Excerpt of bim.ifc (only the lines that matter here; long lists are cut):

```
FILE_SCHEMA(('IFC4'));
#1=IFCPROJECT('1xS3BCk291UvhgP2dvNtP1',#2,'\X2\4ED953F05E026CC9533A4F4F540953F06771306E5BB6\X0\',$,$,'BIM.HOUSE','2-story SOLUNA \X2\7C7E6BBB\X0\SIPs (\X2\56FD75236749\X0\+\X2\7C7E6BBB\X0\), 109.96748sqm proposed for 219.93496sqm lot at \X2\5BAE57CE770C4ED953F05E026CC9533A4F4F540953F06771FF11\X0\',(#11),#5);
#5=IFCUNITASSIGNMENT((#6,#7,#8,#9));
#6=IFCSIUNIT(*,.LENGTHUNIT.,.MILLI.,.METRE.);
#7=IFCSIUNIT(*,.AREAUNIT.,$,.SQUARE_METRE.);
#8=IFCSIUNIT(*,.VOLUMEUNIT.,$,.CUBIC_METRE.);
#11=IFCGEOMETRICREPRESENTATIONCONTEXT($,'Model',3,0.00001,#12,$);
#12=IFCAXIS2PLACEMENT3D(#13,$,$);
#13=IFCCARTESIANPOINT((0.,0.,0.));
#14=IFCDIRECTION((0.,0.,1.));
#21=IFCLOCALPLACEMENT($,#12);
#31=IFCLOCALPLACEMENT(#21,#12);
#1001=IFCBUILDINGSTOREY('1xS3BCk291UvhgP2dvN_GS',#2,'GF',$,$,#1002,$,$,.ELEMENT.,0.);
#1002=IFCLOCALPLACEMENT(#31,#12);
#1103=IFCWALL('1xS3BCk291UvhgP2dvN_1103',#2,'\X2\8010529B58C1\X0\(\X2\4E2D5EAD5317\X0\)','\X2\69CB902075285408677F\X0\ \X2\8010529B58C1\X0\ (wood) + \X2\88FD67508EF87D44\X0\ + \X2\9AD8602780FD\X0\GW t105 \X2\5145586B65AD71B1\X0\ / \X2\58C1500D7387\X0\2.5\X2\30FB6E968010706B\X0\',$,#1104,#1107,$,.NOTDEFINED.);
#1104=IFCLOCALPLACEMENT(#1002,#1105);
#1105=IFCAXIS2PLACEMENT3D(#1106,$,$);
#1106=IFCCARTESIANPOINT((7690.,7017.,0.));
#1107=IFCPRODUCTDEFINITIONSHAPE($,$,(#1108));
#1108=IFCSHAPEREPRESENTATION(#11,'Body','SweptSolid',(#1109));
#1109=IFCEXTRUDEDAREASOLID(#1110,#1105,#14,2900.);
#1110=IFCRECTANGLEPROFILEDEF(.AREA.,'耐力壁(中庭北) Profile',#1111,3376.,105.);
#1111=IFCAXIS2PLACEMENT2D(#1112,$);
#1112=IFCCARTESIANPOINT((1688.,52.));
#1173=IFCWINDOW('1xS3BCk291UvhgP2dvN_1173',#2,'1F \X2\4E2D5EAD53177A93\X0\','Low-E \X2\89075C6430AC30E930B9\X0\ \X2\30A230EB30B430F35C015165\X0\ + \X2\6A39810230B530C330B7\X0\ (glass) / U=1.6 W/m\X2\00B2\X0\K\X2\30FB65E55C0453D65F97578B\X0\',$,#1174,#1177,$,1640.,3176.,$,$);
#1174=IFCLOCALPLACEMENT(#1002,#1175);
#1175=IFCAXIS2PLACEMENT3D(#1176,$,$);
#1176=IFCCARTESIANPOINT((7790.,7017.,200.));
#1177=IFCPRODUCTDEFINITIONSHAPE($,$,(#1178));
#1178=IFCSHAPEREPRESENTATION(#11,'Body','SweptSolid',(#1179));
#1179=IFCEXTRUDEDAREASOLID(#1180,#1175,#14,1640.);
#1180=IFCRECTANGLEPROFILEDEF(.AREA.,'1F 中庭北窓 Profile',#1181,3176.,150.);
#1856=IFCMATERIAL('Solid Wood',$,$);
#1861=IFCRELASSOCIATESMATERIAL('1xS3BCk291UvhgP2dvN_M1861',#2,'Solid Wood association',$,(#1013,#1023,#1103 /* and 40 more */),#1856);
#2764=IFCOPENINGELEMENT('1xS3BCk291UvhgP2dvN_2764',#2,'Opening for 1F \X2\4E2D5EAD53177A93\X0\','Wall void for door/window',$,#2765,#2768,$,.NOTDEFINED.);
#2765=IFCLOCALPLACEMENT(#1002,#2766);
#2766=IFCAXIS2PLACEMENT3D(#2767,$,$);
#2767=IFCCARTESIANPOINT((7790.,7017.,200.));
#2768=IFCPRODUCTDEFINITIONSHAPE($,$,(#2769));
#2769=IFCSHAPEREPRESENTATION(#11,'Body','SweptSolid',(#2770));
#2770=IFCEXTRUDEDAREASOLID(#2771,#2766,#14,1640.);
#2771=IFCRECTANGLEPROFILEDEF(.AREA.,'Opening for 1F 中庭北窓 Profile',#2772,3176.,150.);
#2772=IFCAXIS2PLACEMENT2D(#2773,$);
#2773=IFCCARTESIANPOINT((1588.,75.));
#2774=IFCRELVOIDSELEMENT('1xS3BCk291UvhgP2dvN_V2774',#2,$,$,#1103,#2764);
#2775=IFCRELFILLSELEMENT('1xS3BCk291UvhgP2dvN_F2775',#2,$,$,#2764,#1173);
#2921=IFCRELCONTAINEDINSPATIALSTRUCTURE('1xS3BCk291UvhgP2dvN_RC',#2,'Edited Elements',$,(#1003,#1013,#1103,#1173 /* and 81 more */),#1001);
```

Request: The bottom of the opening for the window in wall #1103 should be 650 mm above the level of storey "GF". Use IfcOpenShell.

```python
import numpy as np
import ifcopenshell
import ifcopenshell.api.geometry
import ifcopenshell.geom
import ifcopenshell.util.element
import ifcopenshell.util.placement
import ifcopenshell.util.shape
import ifcopenshell.util.unit

model = ifcopenshell.open("bim.ifc")
unit_scale = ifcopenshell.util.unit.calculate_unit_scale(model)

window = model.by_guid("1xS3BCk291UvhgP2dvN_1173")
opening = window.FillsVoids[0].RelatingOpeningElement
storey = ifcopenshell.util.element.get_container(window, ifc_class="IfcBuildingStorey")
level = ifcopenshell.util.placement.get_local_placement(storey.ObjectPlacement)[2, 3]

# The opening's origin need not be at the sill, so measure its lowest point.
shape = ifcopenshell.geom.create_shape(ifcopenshell.geom.settings(), opening)
bottom = ifcopenshell.util.shape.get_shape_bottom_elevation(shape, shape.geometry) / unit_scale
dz = level + 0.65 / unit_scale - bottom

shift = np.array([0.0, 0.0, dz])
# The window is not placed relative to its opening, so move both.
for product in (opening, window):
    matrix = ifcopenshell.util.placement.get_local_placement(product.ObjectPlacement)
    matrix[:3, 3] += shift
    ifcopenshell.api.geometry.edit_object_placement(model, product=product, matrix=matrix, is_si=False)

print(f"moved by {dz * unit_scale:+.3f} m")

model.write("bim_rev.ifc")
```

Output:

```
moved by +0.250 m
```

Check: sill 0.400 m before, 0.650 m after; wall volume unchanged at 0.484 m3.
